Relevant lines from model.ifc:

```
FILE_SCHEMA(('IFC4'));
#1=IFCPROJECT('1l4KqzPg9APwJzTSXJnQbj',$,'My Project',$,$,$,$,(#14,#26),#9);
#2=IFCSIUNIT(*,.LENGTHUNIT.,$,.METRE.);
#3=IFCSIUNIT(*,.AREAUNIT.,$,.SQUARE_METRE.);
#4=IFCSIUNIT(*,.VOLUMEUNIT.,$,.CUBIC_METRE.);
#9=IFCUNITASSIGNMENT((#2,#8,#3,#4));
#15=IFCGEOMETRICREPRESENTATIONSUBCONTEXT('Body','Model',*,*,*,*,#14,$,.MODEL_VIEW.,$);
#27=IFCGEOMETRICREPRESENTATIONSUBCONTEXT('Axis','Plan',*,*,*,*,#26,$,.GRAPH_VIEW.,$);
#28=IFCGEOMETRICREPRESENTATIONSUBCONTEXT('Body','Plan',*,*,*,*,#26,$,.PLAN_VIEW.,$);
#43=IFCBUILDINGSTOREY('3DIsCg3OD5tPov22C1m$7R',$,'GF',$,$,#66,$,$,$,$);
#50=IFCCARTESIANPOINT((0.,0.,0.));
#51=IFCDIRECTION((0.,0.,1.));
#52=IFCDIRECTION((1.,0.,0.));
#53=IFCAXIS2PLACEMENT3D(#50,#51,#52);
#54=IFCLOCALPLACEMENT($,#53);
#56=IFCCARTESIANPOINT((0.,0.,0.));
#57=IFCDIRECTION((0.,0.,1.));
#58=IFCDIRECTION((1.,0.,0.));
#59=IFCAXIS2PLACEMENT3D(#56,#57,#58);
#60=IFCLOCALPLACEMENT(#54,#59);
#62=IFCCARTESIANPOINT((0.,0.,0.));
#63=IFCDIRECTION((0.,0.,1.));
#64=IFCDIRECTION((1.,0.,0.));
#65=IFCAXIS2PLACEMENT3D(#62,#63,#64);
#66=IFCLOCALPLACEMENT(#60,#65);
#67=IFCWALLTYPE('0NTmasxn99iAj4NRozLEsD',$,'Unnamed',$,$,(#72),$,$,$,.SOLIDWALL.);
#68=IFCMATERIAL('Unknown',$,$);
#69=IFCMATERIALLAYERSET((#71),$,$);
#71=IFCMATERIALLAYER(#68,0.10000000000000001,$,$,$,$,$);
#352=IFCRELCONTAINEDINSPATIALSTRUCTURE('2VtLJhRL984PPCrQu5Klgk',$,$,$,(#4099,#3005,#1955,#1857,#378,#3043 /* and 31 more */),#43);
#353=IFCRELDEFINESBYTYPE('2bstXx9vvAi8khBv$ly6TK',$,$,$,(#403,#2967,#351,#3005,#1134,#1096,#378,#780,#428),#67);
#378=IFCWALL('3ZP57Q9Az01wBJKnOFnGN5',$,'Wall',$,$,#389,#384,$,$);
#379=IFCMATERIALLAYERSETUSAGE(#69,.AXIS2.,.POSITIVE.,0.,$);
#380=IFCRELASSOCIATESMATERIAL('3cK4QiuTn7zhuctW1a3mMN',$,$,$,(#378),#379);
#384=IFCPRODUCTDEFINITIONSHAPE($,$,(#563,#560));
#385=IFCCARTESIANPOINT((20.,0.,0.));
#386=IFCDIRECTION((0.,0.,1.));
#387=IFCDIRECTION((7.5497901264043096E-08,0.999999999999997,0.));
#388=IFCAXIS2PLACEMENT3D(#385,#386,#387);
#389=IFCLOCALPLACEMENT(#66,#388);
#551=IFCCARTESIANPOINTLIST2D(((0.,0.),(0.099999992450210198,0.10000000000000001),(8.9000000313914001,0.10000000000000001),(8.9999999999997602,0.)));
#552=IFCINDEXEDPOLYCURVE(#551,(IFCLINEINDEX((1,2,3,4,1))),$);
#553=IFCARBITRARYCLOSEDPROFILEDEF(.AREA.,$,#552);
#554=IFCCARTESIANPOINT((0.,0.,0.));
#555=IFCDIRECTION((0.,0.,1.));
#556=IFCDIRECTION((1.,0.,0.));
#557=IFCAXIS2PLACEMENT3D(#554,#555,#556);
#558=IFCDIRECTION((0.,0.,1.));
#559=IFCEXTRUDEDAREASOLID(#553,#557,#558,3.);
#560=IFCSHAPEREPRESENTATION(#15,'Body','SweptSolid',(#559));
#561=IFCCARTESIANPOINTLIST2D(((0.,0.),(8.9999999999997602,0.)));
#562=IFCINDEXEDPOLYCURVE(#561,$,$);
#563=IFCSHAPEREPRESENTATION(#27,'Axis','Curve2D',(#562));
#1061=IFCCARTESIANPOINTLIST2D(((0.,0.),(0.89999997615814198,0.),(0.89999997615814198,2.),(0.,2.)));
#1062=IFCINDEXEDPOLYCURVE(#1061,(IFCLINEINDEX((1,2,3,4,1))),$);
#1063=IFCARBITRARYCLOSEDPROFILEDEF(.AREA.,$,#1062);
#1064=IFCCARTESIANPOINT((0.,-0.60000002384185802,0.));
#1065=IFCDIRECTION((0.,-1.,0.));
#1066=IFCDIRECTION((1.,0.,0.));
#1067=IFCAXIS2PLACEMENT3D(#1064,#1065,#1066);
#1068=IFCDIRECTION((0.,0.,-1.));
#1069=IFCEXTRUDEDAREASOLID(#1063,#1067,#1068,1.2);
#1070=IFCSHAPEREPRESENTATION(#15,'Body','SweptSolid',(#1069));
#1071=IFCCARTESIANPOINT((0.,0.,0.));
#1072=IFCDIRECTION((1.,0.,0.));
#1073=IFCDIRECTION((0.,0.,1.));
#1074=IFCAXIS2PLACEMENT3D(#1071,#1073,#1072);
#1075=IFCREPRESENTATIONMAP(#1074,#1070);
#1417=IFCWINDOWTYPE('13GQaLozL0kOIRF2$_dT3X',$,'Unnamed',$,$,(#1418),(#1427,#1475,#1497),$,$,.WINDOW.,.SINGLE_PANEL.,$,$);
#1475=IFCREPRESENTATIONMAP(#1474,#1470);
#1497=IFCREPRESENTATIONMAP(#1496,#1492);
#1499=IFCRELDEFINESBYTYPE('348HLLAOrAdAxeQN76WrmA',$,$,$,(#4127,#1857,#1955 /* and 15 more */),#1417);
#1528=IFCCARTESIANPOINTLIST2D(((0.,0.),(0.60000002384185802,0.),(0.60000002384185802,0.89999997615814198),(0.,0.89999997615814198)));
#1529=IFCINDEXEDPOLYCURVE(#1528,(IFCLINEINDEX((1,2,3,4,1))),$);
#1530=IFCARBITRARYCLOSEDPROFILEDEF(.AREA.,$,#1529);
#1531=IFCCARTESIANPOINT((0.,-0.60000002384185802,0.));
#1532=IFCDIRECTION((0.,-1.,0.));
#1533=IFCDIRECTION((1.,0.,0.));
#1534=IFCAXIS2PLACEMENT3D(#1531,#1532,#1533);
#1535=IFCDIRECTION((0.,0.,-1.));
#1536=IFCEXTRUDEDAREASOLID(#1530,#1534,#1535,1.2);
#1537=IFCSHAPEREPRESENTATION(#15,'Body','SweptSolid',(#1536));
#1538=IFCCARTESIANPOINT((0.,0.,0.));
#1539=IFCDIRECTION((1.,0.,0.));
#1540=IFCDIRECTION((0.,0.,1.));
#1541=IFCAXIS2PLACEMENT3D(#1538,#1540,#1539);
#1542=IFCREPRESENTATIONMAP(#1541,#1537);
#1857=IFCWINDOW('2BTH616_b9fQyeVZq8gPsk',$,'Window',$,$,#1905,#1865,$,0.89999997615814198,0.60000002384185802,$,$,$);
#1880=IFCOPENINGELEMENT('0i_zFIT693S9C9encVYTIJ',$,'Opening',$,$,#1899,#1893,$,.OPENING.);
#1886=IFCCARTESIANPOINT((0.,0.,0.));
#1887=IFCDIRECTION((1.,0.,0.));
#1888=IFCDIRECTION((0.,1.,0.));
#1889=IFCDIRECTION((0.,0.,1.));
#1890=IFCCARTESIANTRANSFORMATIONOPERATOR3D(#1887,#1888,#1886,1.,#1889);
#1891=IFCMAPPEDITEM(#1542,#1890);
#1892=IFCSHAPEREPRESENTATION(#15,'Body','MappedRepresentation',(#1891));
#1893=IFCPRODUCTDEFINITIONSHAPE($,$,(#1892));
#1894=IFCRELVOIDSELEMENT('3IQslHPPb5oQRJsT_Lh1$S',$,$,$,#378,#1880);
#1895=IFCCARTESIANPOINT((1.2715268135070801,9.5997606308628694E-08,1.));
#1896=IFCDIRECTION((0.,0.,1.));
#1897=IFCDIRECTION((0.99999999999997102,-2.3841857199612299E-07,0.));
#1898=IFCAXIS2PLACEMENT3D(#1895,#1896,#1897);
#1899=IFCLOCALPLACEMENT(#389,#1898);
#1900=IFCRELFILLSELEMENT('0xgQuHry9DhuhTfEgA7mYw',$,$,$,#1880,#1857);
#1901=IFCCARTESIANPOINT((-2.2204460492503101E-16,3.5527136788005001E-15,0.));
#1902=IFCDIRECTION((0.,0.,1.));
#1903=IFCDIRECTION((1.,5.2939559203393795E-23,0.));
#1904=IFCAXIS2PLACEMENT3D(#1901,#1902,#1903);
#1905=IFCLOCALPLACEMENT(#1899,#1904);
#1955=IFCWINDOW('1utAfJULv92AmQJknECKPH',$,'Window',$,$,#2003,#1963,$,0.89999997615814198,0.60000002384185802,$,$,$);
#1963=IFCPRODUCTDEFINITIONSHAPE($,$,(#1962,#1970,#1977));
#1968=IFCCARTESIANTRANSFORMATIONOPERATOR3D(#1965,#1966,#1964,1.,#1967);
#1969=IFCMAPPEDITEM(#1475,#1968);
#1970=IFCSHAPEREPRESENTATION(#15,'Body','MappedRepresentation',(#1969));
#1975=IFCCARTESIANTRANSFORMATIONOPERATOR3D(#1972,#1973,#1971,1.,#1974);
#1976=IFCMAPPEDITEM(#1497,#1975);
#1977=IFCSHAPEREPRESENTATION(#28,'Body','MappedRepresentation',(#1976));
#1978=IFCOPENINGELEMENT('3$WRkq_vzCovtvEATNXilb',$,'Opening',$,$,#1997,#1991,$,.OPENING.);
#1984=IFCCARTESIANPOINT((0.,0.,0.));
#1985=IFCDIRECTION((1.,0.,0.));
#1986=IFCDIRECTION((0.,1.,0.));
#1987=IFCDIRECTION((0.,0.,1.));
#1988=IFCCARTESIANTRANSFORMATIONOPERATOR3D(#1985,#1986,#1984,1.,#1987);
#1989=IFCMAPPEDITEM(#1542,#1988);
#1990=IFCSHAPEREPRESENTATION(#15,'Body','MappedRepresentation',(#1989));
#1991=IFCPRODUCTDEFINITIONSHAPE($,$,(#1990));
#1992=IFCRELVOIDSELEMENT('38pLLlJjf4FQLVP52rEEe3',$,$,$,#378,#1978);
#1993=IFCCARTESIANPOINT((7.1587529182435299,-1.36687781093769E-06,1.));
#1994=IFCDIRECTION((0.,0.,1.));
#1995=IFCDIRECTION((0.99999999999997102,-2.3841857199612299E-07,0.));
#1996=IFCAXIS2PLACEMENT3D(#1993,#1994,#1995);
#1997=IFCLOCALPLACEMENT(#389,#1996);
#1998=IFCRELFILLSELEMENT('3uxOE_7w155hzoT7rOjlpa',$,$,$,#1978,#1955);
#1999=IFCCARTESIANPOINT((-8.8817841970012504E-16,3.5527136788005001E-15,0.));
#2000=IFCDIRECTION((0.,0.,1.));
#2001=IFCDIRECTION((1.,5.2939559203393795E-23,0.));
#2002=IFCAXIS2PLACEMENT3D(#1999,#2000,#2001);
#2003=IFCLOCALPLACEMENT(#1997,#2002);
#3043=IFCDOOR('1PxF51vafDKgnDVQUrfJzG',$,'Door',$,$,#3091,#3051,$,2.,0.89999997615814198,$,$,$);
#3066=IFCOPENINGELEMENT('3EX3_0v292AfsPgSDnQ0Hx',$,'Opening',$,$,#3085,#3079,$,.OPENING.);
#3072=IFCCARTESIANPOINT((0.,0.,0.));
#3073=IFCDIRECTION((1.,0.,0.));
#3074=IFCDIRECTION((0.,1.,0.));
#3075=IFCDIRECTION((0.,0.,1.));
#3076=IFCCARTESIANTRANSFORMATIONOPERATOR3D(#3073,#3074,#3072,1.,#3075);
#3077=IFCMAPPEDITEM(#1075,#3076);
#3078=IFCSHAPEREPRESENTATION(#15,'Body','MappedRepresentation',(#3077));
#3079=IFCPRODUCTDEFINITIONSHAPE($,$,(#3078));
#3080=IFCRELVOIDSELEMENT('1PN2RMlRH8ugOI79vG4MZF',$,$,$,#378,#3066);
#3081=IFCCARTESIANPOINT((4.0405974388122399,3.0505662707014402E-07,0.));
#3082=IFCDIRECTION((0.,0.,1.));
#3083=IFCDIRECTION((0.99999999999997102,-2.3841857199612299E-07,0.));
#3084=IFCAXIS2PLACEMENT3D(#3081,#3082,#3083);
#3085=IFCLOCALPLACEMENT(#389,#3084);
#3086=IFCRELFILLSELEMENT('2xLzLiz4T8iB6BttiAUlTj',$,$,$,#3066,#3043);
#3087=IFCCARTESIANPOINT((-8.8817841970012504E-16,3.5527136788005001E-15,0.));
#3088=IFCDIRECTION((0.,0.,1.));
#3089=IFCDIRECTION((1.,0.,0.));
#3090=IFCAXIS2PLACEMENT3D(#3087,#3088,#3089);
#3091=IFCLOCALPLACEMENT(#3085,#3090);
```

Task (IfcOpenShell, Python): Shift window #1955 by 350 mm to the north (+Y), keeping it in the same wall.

```python
import ifcopenshell
import ifcopenshell.api.geometry
import ifcopenshell.util.placement

model = ifcopenshell.open("model.ifc")

window = model.by_guid("1utAfJULv92AmQJknECKPH")
opening = window.FillsVoids[0].RelatingOpeningElement
wall = opening.VoidsElements[0].RelatingBuildingElement

wall_matrix = ifcopenshell.util.placement.get_local_placement(wall.ObjectPlacement)
shift = wall_matrix[:3, 0] * 0.35
before = ifcopenshell.util.placement.get_local_placement(window.ObjectPlacement)[:3, 3].copy()

# The window is placed relative to its opening, so it follows when the opening moves.
matrix = ifcopenshell.util.placement.get_local_placement(opening.ObjectPlacement)
matrix[:3, 3] += shift
ifcopenshell.api.geometry.edit_object_placement(
    model, product=opening, matrix=matrix, is_si=False, should_transform_children=True
)

after = ifcopenshell.util.placement.get_local_placement(window.ObjectPlacement)[:3, 3]
print("window moved by", (after - before).round(3) + 0.0)

model.write("model_v2.ifc")
```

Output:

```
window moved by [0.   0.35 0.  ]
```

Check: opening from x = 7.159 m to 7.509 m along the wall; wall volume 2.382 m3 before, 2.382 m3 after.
